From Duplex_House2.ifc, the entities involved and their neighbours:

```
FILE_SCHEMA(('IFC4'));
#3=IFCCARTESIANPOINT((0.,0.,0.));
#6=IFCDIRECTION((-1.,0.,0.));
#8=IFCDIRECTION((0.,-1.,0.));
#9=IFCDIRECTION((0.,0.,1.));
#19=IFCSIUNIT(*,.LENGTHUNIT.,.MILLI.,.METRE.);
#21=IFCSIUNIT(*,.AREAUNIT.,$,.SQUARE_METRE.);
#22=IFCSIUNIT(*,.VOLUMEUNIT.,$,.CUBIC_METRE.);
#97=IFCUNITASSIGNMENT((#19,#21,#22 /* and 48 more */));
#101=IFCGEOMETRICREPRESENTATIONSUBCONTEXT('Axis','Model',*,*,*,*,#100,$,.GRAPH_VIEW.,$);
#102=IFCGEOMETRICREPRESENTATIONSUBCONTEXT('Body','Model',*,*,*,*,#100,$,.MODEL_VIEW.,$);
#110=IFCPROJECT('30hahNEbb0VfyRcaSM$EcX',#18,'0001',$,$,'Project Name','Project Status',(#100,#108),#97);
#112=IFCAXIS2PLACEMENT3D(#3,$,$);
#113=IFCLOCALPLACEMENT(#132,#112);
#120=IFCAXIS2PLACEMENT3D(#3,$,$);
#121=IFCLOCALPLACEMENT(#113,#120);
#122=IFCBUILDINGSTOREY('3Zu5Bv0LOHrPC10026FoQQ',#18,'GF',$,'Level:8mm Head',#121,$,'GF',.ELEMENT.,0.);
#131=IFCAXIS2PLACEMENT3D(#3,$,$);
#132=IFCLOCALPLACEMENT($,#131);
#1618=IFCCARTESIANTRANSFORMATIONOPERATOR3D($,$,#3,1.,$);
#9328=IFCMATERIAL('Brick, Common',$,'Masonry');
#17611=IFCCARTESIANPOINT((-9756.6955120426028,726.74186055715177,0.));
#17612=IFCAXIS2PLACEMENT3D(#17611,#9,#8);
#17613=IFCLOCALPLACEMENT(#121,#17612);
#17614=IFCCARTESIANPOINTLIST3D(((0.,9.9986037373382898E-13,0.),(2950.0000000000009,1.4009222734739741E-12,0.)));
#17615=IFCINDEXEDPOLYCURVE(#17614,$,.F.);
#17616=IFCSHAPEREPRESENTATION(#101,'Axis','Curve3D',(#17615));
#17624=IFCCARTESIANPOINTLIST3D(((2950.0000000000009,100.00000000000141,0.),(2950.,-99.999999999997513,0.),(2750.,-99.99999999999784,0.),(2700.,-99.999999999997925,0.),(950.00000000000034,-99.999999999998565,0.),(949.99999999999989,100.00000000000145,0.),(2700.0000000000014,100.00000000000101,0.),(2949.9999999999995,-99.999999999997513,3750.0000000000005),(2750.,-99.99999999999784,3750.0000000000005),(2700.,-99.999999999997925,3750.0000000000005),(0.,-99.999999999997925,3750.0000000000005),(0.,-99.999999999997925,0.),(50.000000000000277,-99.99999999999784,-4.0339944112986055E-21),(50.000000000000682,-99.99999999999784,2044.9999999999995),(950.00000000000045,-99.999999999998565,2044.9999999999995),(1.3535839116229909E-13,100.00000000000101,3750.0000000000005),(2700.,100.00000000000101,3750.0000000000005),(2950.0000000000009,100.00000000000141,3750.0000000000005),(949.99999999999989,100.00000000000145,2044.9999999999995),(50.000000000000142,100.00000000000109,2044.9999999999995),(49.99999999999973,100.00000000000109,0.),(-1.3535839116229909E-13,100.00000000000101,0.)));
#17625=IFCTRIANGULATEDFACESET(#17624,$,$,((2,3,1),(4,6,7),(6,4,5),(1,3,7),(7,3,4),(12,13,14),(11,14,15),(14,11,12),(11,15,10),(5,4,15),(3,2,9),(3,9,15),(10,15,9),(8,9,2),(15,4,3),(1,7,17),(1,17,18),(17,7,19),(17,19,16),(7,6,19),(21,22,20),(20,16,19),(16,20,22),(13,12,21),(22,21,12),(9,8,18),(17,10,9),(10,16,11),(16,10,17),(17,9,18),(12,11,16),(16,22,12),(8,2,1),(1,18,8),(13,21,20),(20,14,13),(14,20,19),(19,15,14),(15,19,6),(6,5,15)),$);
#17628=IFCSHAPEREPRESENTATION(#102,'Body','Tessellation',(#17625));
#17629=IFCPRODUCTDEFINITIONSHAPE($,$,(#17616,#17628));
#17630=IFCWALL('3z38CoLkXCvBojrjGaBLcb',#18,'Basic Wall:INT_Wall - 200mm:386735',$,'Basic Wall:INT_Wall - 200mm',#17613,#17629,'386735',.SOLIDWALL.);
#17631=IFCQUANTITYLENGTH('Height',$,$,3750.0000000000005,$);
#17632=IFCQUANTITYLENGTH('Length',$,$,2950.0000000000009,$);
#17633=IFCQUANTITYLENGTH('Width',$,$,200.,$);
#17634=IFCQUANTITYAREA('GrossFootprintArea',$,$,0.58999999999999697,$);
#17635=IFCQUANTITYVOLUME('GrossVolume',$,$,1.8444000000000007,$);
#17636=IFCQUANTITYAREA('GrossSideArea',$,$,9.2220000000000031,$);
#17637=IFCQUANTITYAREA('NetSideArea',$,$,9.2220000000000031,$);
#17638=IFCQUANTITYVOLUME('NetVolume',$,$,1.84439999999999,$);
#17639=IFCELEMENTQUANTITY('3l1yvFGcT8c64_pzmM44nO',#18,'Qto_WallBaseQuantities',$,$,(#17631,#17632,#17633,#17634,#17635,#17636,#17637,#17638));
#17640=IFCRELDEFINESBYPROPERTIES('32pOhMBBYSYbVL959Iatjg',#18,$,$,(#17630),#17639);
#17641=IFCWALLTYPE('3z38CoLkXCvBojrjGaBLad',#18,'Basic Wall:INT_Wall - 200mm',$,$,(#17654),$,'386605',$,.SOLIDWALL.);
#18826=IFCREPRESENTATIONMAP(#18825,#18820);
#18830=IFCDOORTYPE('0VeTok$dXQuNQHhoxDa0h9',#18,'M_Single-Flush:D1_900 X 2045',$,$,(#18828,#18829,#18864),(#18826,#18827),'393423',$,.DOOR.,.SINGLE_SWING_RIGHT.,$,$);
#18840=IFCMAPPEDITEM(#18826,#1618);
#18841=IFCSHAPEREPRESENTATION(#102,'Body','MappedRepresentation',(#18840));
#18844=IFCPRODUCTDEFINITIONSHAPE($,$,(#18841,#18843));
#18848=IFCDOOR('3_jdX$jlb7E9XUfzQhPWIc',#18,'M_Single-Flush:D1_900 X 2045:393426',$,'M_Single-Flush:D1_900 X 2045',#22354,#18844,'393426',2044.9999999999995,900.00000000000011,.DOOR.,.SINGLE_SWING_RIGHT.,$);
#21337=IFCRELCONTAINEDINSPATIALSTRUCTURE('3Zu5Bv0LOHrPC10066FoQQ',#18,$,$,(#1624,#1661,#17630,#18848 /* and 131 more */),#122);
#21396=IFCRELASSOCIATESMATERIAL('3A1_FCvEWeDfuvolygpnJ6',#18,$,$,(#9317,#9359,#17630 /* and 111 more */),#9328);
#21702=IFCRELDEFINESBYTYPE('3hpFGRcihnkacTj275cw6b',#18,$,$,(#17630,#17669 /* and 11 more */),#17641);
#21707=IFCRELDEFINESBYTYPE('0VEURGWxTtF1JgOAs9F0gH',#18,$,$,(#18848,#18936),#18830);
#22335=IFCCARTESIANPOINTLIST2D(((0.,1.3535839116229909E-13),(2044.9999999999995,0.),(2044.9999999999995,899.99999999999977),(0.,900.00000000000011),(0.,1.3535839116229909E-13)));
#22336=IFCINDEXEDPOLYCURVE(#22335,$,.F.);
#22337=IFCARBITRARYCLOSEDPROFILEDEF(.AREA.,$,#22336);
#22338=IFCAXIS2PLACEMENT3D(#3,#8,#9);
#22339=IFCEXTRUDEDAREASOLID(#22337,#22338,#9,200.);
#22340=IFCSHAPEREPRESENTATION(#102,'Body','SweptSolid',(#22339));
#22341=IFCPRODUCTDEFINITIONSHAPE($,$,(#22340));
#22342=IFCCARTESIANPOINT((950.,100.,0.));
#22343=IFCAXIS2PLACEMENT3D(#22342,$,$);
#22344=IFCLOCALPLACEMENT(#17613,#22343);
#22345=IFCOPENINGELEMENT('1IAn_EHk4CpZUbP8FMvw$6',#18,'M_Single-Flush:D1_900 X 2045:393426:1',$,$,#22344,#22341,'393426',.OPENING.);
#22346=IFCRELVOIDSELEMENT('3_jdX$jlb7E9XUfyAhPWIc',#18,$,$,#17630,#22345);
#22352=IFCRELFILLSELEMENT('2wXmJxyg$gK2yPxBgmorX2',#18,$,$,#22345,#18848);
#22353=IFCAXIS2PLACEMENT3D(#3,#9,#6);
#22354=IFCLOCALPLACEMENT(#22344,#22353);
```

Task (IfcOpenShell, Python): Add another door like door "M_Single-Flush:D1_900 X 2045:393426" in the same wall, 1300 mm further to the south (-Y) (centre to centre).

```python
import ifcopenshell
import ifcopenshell.api.feature
import ifcopenshell.api.geometry
import ifcopenshell.api.pset
import ifcopenshell.api.root
import ifcopenshell.geom
import ifcopenshell.util.element
import ifcopenshell.util.placement
import ifcopenshell.util.shape
import ifcopenshell.util.unit

model = ifcopenshell.open("Duplex_House2.ifc")
area_scale = ifcopenshell.util.unit.calculate_unit_scale(model, "AREAUNIT")
volume_scale = ifcopenshell.util.unit.calculate_unit_scale(model, "VOLUMEUNIT")
settings = ifcopenshell.geom.settings()


def volume(element):
    """Net volume in cubic metres, openings subtracted."""
    shape = ifcopenshell.geom.create_shape(settings, element)
    return ifcopenshell.util.shape.get_volume(shape.geometry)


def reuse_history(source, copy):
    """copy_class also copies each property set's owner history, people and application; keep the originals."""
    for rel in copy.IsDefinedBy:
        if rel.is_a("IfcRelDefinesByProperties") and (history := rel.RelatingPropertyDefinition.OwnerHistory):
            rel.RelatingPropertyDefinition.OwnerHistory = source.OwnerHistory
            ifcopenshell.util.element.remove_deep2(model, history)


door = model.by_guid("3_jdX$jlb7E9XUfzQhPWIc")
opening = door.FillsVoids[0].RelatingOpeningElement
wall = opening.VoidsElements[0].RelatingBuildingElement
before = volume(wall)
shift = ifcopenshell.util.placement.get_local_placement(wall.ObjectPlacement)[:3, 0] * 1300.0

# copy_class copies the void relationship, type, container and properties, but no geometry.
new_opening = ifcopenshell.api.root.copy_class(model, product=opening)
new_opening.Representation = ifcopenshell.util.element.copy_deep(
    model, opening.Representation, exclude=["IfcGeometricRepresentationContext", "IfcRepresentationMap"]
)
new_opening.Name = "M_Single-Flush:D1_900 X 2045"
new_opening.Tag = None
reuse_history(opening, new_opening)
new_door = ifcopenshell.api.root.copy_class(model, product=door)
new_door.Representation = ifcopenshell.util.element.copy_deep(
    model, door.Representation, exclude=["IfcGeometricRepresentationContext", "IfcRepresentationMap"]
)
new_door.Name = "M_Single-Flush:D1_900 X 2045"
new_door.Tag = None
reuse_history(door, new_door)
ifcopenshell.api.feature.add_filling(model, opening=new_opening, element=new_door)

for old, new in ((opening, new_opening), (door, new_door)):
    matrix = ifcopenshell.util.placement.get_local_placement(old.ObjectPlacement)
    matrix[:3, 3] += shift
    ifcopenshell.api.geometry.edit_object_placement(model, product=new, matrix=matrix, is_si=False)

after = volume(wall)
thickness = 0.2  # wall thickness in metres

# Update the wall's stored quantities.
qto = model.by_id(ifcopenshell.util.element.get_pset(wall, "Qto_WallBaseQuantities", should_inherit=False)["id"])
ifcopenshell.api.pset.edit_qto(model, qto=qto, properties={
    "NetSideArea": after / thickness / area_scale,
    "NetVolume": after / volume_scale,
})

print(f"wall volume {before:.3f} -> {after:.3f} m3")

model.write("Duplex_House2_updated.ifc")
```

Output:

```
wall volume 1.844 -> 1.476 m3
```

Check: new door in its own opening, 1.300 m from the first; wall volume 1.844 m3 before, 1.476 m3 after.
